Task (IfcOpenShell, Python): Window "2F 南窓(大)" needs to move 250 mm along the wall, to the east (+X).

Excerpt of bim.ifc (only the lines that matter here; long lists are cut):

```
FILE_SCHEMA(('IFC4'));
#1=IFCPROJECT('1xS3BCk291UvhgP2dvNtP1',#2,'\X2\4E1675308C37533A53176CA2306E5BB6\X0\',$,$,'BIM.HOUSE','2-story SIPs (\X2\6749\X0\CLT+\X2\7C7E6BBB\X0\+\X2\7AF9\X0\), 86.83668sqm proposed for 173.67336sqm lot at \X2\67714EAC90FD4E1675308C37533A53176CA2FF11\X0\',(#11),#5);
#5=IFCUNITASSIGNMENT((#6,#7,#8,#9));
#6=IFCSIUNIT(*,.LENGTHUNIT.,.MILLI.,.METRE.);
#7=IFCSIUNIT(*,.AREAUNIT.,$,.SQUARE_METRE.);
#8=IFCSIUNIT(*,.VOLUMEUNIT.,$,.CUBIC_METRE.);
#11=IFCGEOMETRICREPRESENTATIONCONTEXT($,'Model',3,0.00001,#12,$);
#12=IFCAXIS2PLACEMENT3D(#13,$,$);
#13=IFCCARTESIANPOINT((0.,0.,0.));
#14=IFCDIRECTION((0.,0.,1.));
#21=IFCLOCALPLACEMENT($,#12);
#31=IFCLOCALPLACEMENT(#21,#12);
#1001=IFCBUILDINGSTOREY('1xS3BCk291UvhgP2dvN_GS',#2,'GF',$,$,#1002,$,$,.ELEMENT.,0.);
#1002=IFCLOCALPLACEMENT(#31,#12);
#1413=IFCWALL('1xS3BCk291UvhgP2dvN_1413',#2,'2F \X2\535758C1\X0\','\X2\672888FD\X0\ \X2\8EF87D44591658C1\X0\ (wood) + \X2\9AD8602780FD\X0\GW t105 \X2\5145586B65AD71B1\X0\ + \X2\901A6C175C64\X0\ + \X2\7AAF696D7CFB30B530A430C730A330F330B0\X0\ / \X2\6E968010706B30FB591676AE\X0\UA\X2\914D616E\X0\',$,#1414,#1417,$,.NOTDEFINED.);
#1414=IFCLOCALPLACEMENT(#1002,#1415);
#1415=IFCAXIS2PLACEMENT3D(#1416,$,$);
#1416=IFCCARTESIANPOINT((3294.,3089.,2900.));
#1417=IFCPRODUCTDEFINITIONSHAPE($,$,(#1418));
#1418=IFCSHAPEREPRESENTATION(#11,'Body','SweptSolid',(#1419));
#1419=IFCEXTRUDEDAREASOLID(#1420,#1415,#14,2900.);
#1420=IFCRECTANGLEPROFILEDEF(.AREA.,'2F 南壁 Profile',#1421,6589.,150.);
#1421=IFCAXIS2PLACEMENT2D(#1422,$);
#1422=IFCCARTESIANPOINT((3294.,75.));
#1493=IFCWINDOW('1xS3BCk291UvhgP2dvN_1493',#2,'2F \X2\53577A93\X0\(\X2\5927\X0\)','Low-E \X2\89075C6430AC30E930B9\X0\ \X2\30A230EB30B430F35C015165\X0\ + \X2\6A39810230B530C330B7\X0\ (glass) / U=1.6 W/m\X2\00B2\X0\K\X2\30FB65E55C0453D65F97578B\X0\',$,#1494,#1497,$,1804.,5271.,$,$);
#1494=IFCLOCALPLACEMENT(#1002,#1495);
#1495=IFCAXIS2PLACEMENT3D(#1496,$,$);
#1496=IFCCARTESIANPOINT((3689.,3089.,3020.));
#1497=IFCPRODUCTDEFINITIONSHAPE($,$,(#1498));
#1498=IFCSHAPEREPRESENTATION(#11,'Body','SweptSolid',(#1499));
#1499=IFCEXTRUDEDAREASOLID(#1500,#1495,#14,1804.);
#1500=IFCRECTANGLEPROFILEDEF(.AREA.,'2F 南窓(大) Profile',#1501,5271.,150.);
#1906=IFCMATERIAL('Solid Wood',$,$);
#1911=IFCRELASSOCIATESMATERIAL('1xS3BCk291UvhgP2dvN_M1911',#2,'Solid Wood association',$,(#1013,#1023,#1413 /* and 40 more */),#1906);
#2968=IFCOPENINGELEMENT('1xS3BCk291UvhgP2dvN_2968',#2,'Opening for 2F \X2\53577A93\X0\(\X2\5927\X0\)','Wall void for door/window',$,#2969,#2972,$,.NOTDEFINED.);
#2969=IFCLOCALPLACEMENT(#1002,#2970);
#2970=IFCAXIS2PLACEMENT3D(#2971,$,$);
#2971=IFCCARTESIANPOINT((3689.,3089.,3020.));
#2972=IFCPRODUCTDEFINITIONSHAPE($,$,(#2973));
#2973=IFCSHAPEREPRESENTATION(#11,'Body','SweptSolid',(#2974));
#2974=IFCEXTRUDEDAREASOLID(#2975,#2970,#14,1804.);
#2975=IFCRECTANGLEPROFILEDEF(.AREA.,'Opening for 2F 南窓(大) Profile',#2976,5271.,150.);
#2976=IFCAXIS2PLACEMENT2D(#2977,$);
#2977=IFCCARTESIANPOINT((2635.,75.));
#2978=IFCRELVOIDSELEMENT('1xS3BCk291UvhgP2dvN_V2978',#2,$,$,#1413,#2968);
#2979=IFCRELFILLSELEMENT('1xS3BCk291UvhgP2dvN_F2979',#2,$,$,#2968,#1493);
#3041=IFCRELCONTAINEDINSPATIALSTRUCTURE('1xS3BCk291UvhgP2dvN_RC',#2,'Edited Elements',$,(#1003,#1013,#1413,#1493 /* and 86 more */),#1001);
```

```python
import ifcopenshell
import ifcopenshell.api.geometry
import ifcopenshell.util.placement
import ifcopenshell.util.unit

model = ifcopenshell.open("bim.ifc")
unit_scale = ifcopenshell.util.unit.calculate_unit_scale(model)

window = model.by_guid("1xS3BCk291UvhgP2dvN_1493")
opening = window.FillsVoids[0].RelatingOpeningElement
wall = opening.VoidsElements[0].RelatingBuildingElement

wall_matrix = ifcopenshell.util.placement.get_local_placement(wall.ObjectPlacement)
shift = wall_matrix[:3, 0] * 0.25 / unit_scale
before = ifcopenshell.util.placement.get_local_placement(window.ObjectPlacement)[:3, 3].copy()

# The window is not placed relative to its opening, so move both.
for product in (opening, window):
    matrix = ifcopenshell.util.placement.get_local_placement(product.ObjectPlacement)
    matrix[:3, 3] += shift
    ifcopenshell.api.geometry.edit_object_placement(model, product=product, matrix=matrix, is_si=False)

after = ifcopenshell.util.placement.get_local_placement(window.ObjectPlacement)[:3, 3]
print("window moved by", (after - before).round(3) + 0.0)

model.write("bim-out.ifc")
```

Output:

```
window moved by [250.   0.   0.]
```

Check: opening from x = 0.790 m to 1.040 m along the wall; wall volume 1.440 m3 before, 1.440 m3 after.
